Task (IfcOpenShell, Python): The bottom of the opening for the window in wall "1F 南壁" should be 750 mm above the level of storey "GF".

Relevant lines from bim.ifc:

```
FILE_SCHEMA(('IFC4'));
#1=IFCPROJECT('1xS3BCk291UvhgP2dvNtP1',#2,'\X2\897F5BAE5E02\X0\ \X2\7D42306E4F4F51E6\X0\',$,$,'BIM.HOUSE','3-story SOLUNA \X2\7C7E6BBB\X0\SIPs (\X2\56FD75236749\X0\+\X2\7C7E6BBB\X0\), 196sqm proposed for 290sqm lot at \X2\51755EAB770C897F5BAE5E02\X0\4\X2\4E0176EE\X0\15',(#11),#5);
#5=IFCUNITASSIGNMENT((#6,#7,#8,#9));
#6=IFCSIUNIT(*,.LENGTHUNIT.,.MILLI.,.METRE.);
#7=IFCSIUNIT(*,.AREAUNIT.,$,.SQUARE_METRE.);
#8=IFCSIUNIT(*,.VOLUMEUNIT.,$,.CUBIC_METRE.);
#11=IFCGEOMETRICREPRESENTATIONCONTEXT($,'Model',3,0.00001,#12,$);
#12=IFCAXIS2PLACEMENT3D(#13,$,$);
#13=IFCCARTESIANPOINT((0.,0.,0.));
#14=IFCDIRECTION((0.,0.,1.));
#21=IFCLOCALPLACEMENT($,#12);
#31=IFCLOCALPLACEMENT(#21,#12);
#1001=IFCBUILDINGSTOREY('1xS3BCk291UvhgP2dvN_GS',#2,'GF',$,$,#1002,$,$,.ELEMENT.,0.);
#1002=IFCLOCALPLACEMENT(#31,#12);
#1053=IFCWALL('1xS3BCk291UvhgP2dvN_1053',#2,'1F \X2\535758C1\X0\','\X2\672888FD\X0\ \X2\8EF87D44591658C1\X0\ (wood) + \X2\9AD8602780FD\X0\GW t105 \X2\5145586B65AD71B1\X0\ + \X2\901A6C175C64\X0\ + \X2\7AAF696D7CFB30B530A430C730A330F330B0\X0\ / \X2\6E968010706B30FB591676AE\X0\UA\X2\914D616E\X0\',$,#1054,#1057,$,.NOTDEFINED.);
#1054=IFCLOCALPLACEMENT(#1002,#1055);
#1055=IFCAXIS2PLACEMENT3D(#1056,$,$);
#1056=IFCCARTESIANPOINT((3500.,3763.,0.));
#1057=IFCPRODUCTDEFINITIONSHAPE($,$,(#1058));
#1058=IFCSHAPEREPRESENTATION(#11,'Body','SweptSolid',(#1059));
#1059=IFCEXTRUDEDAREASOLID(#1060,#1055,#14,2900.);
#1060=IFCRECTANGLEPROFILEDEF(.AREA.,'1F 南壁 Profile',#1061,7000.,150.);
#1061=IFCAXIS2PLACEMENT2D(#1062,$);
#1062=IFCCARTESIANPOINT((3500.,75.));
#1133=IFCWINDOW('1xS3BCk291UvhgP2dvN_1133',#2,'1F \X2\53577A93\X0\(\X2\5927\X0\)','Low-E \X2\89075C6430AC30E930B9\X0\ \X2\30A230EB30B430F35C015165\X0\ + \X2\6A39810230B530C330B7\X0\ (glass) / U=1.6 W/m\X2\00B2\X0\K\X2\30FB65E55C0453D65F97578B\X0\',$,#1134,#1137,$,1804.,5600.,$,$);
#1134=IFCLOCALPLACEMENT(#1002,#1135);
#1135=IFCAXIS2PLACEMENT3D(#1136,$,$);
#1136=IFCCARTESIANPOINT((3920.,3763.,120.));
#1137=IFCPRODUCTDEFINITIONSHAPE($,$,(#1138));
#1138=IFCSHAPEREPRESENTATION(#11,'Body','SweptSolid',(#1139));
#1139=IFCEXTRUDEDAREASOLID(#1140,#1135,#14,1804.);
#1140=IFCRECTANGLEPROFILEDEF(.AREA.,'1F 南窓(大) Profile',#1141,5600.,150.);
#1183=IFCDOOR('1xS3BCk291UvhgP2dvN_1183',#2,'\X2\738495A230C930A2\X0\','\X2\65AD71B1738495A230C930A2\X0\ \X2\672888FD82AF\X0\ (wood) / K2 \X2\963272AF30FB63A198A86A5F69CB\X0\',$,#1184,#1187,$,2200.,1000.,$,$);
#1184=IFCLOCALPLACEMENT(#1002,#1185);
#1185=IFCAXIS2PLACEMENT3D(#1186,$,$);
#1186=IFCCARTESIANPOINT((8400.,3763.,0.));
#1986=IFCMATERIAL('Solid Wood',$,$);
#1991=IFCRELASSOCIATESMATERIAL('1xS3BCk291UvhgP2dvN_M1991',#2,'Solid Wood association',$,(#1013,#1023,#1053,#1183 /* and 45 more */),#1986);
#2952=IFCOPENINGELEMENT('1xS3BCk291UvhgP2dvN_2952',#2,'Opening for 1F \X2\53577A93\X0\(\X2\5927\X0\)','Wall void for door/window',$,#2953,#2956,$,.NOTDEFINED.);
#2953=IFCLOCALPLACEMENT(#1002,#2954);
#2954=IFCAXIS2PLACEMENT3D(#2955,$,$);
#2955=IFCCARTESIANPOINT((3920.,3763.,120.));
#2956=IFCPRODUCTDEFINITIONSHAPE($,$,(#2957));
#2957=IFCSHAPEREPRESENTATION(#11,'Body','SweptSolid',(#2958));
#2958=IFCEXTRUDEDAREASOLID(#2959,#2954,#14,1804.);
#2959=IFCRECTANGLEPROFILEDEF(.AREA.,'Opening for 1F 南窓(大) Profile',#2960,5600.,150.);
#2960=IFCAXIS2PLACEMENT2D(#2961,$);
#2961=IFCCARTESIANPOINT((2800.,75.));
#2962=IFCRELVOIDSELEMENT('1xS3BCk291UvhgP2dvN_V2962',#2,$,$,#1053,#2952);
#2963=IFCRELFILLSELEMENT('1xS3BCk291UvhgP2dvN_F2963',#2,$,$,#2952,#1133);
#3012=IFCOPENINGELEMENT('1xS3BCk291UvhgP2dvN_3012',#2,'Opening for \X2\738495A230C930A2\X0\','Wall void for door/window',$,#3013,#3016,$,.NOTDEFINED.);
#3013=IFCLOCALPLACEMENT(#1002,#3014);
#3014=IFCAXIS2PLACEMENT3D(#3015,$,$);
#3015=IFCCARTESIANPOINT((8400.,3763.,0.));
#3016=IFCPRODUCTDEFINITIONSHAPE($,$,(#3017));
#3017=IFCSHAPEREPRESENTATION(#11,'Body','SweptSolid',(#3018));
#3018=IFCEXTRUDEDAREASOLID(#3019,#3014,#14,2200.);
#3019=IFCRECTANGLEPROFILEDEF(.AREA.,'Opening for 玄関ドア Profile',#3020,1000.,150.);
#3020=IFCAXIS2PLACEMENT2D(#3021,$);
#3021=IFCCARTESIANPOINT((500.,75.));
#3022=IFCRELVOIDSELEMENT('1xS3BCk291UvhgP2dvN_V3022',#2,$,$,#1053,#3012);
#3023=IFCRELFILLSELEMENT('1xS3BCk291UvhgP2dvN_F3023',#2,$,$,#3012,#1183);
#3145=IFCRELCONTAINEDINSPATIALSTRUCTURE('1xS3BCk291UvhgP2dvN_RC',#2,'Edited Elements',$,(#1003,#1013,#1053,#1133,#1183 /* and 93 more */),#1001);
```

```python
import numpy as np
import ifcopenshell
import ifcopenshell.api.geometry
import ifcopenshell.geom
import ifcopenshell.util.element
import ifcopenshell.util.placement
import ifcopenshell.util.shape
import ifcopenshell.util.unit

model = ifcopenshell.open("bim.ifc")
unit_scale = ifcopenshell.util.unit.calculate_unit_scale(model)

window = model.by_id(1133)
opening = window.FillsVoids[0].RelatingOpeningElement
storey = ifcopenshell.util.element.get_container(window, ifc_class="IfcBuildingStorey")
level = ifcopenshell.util.placement.get_local_placement(storey.ObjectPlacement)[2, 3]

# The opening's origin need not be at the sill, so measure its lowest point.
shape = ifcopenshell.geom.create_shape(ifcopenshell.geom.settings(), opening)
bottom = ifcopenshell.util.shape.get_shape_bottom_elevation(shape, shape.geometry) / unit_scale
dz = level + 0.75 / unit_scale - bottom

shift = np.array([0.0, 0.0, dz])
# The window is not placed relative to its opening, so move both.
for product in (opening, window):
    matrix = ifcopenshell.util.placement.get_local_placement(product.ObjectPlacement)
    matrix[:3, 3] += shift
    ifcopenshell.api.geometry.edit_object_placement(model, product=product, matrix=matrix, is_si=False)

print(f"moved by {dz * unit_scale:+.3f} m")

model.write("bim_rev.ifc")
```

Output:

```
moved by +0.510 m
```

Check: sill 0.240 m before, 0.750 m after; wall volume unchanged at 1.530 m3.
